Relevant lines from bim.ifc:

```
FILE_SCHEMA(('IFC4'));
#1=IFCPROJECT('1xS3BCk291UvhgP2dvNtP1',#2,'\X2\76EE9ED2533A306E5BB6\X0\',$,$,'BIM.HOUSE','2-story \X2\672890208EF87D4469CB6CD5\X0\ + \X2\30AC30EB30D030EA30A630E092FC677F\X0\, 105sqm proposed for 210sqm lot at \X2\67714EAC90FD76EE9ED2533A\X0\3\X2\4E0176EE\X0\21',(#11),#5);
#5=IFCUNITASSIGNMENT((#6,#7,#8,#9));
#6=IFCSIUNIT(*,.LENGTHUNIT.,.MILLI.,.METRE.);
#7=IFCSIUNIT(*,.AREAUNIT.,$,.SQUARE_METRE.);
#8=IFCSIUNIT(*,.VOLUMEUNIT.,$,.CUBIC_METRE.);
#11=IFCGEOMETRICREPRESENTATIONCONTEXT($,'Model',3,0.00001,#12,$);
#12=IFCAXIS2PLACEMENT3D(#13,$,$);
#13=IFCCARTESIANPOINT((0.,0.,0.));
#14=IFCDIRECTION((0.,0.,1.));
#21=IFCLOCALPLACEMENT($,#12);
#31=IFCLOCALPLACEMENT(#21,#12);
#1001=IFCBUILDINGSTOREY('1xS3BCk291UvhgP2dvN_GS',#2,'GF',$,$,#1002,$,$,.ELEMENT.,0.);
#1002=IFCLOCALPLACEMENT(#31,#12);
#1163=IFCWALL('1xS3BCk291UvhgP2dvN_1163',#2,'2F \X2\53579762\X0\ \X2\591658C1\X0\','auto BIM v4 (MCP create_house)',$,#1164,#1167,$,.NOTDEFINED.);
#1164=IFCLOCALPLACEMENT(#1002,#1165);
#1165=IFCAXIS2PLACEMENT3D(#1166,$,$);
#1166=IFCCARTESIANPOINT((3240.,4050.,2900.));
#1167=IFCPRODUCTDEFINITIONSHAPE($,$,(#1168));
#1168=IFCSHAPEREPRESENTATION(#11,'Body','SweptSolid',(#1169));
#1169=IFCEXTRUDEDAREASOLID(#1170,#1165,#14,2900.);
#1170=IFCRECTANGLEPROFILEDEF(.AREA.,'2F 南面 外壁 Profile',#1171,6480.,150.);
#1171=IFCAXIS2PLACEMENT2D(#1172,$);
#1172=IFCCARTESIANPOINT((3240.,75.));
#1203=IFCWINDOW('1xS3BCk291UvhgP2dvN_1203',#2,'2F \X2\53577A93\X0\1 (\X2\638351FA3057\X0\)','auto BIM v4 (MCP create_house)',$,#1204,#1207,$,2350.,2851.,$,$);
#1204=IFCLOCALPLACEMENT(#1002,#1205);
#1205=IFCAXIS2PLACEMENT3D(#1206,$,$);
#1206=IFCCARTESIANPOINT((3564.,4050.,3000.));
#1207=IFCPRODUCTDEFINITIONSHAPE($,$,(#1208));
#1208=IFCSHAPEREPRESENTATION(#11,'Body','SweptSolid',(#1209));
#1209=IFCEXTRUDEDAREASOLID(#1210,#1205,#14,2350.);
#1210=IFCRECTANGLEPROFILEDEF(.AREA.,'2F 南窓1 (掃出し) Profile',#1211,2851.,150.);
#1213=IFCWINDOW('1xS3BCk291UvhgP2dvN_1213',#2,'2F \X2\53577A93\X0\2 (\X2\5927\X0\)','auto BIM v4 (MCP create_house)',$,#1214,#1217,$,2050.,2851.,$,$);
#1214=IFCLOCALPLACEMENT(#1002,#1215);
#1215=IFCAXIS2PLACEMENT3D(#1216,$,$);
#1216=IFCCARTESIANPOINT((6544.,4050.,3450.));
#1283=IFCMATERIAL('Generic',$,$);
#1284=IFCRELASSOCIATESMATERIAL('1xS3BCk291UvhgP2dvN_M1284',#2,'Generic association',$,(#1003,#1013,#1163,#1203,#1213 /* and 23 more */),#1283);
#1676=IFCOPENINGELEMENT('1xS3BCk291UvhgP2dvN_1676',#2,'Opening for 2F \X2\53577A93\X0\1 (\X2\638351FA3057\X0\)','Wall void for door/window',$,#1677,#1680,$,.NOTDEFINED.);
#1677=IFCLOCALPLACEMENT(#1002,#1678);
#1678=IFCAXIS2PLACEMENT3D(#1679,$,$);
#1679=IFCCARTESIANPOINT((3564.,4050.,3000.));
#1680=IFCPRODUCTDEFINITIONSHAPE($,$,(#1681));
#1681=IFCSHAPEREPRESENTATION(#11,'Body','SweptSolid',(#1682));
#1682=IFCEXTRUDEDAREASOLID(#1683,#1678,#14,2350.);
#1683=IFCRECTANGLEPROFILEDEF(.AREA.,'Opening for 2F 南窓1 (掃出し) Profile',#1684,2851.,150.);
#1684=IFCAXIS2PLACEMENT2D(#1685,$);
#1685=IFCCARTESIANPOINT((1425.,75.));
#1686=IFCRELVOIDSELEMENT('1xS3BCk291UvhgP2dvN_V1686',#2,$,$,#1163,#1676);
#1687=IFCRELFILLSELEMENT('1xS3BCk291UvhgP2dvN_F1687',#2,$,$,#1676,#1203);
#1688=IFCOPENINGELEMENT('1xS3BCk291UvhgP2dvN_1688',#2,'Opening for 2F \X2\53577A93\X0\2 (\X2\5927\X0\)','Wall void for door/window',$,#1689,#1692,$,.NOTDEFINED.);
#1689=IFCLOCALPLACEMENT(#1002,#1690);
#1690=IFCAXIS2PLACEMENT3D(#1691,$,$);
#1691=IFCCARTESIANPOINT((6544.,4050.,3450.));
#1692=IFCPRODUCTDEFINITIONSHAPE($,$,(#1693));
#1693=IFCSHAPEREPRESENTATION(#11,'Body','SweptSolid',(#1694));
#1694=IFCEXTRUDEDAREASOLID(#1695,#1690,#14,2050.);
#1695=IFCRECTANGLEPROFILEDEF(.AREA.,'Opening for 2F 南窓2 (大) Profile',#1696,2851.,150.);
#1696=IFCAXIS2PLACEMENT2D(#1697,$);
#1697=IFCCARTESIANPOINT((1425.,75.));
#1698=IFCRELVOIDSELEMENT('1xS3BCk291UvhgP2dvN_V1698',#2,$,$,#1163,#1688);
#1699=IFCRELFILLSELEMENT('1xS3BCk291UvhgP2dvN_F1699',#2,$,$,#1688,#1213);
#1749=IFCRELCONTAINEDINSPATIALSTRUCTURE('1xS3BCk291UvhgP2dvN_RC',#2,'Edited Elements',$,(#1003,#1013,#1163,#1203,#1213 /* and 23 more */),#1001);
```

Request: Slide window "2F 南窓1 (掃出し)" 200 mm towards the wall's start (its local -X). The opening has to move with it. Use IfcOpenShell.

```python
import ifcopenshell
import ifcopenshell.api.geometry
import ifcopenshell.util.placement

model = ifcopenshell.open("bim.ifc")

window = model.by_guid("1xS3BCk291UvhgP2dvN_1203")
opening = window.FillsVoids[0].RelatingOpeningElement
wall = opening.VoidsElements[0].RelatingBuildingElement

wall_matrix = ifcopenshell.util.placement.get_local_placement(wall.ObjectPlacement)
shift = wall_matrix[:3, 0] * -200.0
before = ifcopenshell.util.placement.get_local_placement(window.ObjectPlacement)[:3, 3].copy()

# The window is not placed relative to its opening, so move both.
for product in (opening, window):
    matrix = ifcopenshell.util.placement.get_local_placement(product.ObjectPlacement)
    matrix[:3, 3] += shift
    ifcopenshell.api.geometry.edit_object_placement(model, product=product, matrix=matrix, is_si=False)

after = ifcopenshell.util.placement.get_local_placement(window.ObjectPlacement)[:3, 3]
print("window moved by", (after - before).round(3) + 0.0)

model.write("bim_rev.ifc")
```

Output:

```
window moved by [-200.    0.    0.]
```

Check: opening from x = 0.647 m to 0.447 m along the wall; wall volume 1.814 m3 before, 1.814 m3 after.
